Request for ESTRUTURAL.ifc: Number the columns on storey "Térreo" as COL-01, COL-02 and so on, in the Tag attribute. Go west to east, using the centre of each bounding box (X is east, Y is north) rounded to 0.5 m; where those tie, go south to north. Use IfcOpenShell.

First a look at what the model holds.

```python
import ifcopenshell
import ifcopenshell.util.element
import ifcopenshell.util.placement

model = ifcopenshell.open("ESTRUTURAL.ifc")
print(model.schema)
storey = next(s for s in model.by_type("IfcBuildingStorey") if s.Name == "Térreo")
columns = [e for e in ifcopenshell.util.element.get_decomposition(storey) if e.is_a("IfcColumn")]
for e in sorted(columns, key=lambda e: e.id()):
    origin = ifcopenshell.util.placement.get_local_placement(e.ObjectPlacement)[:3, 3]
    print(e.id(), e.Tag, e.Name, origin.round(2) + 0.0, sep=" | ")
```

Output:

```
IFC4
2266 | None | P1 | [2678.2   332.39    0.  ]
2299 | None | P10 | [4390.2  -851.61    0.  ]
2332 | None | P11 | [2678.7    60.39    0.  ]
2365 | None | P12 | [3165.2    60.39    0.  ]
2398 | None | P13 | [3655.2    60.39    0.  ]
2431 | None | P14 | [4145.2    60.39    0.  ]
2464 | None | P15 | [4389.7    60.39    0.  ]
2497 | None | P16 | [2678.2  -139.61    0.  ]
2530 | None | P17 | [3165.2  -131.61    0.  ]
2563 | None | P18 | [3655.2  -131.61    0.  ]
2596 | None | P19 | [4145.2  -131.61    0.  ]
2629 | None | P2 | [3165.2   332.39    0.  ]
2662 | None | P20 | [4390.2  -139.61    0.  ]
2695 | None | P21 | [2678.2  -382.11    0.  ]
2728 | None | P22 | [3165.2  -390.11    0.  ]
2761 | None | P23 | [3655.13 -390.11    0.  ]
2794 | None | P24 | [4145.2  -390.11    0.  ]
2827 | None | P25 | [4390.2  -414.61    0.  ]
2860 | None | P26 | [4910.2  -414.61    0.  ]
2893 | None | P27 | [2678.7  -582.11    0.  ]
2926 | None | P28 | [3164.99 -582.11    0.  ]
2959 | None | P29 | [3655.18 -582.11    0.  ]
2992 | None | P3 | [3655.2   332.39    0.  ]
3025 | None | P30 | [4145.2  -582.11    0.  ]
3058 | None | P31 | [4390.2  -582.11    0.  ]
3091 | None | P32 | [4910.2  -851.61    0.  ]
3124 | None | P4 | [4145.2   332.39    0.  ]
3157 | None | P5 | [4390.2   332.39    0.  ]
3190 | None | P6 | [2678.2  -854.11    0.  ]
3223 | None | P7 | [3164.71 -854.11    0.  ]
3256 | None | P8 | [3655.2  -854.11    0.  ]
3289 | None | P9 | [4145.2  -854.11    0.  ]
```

```python
import ifcopenshell
import ifcopenshell.geom
import ifcopenshell.util.element
import ifcopenshell.util.shape

model = ifcopenshell.open("ESTRUTURAL.ifc")
settings = ifcopenshell.geom.settings()
settings.set("use-world-coords", True)


def centre(element):
    shape = ifcopenshell.geom.create_shape(settings, element)
    return ifcopenshell.util.shape.get_bbox_centroid(shape.geometry)


storey = next(s for s in model.by_type("IfcBuildingStorey") if s.Name == "Térreo")
columns = [e for e in ifcopenshell.util.element.get_decomposition(storey) if e.is_a("IfcColumn")]

# Insertion points can sit at a corner or the storey origin, so sort by the geometry (in metres).
centres = {e: centre(e) for e in columns}
columns.sort(key=lambda e: (round(centres[e][0] / 0.5), centres[e][1]))

for i, e in enumerate(columns, start=1):
    number = f"COL-{i:02d}"
    e.Tag = number
    print(e.id(), number)

model.write("ESTRUTURAL_rev.ifc")
```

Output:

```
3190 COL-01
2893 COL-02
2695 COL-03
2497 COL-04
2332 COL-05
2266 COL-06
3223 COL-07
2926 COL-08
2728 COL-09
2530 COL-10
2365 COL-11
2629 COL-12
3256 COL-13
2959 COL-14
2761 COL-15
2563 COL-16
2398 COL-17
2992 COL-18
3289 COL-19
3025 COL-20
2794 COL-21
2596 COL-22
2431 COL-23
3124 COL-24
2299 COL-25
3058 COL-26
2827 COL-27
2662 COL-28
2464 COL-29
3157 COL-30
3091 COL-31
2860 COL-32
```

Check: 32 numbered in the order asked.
